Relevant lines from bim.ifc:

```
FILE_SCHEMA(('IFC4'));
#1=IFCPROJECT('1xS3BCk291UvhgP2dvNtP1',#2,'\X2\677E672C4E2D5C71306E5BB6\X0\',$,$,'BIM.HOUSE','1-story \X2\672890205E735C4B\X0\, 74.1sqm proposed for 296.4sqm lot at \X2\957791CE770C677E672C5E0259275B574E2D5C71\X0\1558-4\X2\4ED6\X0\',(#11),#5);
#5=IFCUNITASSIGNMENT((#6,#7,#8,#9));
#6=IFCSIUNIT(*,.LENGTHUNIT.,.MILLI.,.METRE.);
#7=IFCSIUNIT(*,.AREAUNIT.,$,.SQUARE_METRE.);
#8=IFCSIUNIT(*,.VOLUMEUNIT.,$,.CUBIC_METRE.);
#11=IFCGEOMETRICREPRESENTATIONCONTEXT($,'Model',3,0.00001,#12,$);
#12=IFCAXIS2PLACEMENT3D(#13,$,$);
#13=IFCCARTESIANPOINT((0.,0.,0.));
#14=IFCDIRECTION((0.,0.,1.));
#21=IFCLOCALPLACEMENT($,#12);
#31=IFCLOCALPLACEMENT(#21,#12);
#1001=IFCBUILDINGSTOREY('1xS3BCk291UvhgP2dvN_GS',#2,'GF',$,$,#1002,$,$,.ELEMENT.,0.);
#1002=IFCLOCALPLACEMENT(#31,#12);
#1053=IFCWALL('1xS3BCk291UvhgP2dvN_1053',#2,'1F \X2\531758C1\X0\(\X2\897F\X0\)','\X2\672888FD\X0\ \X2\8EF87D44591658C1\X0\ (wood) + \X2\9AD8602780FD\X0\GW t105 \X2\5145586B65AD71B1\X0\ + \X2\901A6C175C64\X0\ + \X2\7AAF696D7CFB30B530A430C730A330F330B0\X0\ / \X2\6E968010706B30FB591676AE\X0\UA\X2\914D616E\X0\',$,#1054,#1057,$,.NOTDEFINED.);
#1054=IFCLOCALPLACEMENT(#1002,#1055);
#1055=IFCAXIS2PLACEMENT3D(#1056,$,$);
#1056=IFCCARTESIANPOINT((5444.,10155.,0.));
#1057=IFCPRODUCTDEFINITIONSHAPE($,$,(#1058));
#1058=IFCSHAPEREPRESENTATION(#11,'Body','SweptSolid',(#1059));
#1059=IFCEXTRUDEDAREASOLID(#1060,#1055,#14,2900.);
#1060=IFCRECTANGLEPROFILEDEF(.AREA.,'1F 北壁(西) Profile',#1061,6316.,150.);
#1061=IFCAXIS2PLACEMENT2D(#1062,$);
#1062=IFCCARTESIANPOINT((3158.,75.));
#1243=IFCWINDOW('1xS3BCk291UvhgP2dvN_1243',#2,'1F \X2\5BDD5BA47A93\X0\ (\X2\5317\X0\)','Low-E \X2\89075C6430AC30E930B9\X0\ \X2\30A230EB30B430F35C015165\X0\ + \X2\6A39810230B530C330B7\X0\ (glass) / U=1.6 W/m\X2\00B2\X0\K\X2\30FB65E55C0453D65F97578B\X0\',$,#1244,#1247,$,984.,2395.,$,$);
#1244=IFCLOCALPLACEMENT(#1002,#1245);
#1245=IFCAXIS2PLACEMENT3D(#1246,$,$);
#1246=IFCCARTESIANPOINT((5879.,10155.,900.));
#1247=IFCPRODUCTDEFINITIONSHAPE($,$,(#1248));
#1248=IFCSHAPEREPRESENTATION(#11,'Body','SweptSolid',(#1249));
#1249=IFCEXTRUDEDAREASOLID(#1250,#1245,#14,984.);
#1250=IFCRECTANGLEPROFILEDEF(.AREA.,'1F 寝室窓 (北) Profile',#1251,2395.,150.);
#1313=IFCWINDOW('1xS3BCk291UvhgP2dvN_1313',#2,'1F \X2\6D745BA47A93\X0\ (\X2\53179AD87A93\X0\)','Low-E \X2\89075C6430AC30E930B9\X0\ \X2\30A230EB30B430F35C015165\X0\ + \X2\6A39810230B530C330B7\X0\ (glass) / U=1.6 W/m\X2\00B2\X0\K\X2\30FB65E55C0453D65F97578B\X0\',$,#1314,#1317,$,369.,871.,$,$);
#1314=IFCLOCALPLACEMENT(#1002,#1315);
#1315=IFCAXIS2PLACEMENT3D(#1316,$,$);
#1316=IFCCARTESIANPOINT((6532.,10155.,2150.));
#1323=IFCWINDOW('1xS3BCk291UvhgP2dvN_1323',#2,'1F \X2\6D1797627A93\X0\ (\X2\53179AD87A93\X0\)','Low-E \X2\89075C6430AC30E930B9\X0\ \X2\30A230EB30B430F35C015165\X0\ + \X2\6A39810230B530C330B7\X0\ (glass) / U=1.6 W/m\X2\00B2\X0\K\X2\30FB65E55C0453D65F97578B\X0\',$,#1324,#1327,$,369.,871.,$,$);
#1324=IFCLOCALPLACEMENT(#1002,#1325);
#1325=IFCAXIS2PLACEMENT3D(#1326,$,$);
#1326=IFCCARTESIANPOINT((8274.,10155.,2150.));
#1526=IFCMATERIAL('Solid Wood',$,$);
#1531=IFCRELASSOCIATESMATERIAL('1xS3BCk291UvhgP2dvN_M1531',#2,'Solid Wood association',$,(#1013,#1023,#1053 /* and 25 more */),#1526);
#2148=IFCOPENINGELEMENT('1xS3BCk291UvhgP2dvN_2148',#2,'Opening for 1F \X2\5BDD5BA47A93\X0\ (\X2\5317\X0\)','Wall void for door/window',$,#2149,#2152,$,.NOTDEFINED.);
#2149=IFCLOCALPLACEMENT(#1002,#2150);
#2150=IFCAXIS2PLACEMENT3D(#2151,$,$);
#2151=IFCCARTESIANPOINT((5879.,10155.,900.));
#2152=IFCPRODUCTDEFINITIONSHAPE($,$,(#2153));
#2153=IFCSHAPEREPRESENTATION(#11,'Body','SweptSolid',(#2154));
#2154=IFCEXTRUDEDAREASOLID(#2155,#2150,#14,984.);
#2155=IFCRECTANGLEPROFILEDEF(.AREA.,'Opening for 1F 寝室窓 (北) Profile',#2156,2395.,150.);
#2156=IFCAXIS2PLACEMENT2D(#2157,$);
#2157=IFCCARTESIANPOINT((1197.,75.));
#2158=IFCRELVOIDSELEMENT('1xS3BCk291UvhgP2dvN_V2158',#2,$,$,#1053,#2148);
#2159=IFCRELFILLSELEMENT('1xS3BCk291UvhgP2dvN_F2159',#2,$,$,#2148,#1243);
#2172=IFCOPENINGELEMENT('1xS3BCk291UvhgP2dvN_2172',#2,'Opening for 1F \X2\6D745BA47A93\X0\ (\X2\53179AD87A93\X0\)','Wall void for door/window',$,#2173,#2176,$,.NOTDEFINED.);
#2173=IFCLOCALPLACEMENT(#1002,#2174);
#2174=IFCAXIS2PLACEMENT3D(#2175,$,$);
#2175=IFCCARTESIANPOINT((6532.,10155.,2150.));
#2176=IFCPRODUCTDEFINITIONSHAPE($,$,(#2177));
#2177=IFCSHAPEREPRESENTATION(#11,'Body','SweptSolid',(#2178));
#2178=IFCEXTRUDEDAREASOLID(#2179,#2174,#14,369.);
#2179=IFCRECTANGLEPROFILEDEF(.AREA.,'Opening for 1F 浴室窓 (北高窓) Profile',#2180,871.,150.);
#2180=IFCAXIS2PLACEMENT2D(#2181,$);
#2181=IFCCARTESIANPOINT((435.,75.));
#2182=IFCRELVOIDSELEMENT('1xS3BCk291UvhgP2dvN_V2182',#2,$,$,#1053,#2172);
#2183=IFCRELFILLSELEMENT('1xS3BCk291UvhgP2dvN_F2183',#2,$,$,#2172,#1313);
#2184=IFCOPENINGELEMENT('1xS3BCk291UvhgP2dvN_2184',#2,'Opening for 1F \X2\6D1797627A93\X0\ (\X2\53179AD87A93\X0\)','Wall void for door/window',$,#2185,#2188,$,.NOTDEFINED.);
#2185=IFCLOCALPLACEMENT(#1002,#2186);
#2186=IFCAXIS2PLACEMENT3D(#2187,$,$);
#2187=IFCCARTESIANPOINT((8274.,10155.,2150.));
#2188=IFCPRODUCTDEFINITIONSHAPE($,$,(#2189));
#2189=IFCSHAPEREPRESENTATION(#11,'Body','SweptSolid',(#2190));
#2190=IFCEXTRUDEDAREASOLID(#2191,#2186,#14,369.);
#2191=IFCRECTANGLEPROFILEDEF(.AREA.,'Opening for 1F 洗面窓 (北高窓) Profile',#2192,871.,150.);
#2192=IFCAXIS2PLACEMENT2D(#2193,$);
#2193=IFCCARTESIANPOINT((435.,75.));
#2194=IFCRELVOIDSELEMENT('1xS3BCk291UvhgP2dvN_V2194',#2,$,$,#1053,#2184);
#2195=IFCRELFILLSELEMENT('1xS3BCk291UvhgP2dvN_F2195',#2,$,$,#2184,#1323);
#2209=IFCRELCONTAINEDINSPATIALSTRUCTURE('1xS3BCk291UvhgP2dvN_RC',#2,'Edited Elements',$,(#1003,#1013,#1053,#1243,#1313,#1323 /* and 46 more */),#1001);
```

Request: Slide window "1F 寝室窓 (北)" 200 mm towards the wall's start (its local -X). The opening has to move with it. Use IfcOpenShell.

```python
import ifcopenshell
import ifcopenshell.api.geometry
import ifcopenshell.util.placement

model = ifcopenshell.open("bim.ifc")

window = model.by_id(1243)
opening = window.FillsVoids[0].RelatingOpeningElement
wall = opening.VoidsElements[0].RelatingBuildingElement

wall_matrix = ifcopenshell.util.placement.get_local_placement(wall.ObjectPlacement)
shift = wall_matrix[:3, 0] * -200.0
before = ifcopenshell.util.placement.get_local_placement(window.ObjectPlacement)[:3, 3].copy()

# The window is not placed relative to its opening, so move both.
for product in (opening, window):
    matrix = ifcopenshell.util.placement.get_local_placement(product.ObjectPlacement)
    matrix[:3, 3] += shift
    ifcopenshell.api.geometry.edit_object_placement(model, product=product, matrix=matrix, is_si=False)

after = ifcopenshell.util.placement.get_local_placement(window.ObjectPlacement)[:3, 3]
print("window moved by", (after - before).round(3) + 0.0)

model.write("bim_rev.ifc")
```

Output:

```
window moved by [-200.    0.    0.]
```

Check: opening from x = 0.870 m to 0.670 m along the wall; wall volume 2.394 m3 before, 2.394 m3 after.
